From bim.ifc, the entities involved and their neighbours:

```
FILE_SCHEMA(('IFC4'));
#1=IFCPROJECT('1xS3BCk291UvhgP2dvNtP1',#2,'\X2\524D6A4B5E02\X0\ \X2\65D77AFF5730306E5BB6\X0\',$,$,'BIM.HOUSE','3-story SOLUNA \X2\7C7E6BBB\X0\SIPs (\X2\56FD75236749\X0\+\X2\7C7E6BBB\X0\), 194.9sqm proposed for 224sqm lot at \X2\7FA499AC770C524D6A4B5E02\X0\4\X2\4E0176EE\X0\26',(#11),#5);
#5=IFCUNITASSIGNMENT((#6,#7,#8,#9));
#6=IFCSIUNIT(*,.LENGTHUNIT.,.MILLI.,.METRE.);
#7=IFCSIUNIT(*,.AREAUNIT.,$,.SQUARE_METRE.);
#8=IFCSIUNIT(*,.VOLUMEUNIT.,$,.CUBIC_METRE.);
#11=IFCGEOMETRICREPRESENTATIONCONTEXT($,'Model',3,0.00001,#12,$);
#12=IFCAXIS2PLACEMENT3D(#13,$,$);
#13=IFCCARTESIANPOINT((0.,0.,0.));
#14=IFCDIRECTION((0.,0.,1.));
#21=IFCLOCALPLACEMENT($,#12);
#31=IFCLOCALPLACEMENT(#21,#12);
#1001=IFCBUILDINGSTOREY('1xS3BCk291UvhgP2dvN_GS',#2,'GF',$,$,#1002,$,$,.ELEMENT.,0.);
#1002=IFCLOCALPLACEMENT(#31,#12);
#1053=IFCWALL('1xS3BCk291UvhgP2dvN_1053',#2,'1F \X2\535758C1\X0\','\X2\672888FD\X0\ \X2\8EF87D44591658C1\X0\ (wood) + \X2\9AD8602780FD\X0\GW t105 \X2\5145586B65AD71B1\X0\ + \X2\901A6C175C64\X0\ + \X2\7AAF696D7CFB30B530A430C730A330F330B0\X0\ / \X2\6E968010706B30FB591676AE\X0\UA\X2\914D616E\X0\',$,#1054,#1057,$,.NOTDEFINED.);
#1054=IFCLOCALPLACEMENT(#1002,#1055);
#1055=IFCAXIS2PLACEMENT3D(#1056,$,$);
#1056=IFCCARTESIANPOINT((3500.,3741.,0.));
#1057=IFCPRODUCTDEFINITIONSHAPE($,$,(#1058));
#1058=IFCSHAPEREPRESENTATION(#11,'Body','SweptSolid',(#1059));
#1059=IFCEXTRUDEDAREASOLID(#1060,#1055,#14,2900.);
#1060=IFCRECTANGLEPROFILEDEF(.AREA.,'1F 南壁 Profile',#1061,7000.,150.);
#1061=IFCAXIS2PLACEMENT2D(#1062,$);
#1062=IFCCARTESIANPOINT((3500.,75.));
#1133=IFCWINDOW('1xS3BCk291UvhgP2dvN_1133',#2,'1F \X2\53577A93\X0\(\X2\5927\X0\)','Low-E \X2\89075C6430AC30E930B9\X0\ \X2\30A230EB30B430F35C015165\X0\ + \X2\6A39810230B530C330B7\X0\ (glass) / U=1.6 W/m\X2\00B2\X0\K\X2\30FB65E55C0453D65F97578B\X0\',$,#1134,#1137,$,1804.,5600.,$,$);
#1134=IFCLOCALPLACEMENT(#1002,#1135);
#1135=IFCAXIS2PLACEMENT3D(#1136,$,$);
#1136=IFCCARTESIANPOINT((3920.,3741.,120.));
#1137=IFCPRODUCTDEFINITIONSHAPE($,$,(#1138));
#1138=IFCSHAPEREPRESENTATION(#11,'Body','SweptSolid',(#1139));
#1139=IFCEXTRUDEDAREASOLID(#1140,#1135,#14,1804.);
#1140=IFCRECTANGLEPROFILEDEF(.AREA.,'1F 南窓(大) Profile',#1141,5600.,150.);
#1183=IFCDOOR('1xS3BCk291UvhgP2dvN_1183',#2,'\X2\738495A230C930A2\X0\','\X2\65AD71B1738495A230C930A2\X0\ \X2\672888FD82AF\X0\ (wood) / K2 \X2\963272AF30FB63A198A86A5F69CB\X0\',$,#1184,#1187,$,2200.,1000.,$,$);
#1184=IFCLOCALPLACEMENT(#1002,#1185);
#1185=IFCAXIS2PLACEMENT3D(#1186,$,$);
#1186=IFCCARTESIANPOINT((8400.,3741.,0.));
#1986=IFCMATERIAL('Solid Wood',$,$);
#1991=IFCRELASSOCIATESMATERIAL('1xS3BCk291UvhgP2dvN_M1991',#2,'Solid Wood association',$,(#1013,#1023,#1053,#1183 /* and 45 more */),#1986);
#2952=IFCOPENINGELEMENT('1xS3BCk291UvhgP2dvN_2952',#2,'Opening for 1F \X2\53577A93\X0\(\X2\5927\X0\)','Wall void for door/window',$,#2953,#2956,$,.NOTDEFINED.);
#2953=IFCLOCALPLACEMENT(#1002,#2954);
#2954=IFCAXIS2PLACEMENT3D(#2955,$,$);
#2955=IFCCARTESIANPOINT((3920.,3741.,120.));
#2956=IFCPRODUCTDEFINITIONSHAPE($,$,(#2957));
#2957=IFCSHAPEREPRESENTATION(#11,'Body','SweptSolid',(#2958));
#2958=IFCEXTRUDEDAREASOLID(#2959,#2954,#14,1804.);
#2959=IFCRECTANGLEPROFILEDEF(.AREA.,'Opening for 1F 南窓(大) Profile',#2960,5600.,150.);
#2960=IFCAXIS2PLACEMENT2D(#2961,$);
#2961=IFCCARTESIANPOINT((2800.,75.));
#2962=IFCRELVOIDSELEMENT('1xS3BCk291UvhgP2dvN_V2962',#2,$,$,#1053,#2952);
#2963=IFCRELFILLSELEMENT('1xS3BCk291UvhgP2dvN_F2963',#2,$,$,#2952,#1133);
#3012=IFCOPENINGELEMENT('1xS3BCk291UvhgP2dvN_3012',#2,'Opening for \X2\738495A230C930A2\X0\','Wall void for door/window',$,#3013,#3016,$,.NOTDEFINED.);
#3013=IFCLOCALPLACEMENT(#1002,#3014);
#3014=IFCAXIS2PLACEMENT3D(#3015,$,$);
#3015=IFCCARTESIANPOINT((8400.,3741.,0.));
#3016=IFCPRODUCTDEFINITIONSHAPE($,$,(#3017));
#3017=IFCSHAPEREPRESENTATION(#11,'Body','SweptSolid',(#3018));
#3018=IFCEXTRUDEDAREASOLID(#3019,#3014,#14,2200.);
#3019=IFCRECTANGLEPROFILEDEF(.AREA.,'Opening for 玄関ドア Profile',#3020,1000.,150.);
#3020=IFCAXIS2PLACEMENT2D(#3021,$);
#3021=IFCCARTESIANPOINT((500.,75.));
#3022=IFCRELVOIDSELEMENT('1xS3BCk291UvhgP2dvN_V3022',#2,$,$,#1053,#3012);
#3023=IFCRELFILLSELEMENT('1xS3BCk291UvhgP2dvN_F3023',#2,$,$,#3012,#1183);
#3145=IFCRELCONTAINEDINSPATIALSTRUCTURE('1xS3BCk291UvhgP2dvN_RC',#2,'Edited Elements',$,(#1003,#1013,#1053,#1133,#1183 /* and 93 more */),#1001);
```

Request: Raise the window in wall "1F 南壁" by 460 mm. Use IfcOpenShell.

```python
import numpy as np
import ifcopenshell
import ifcopenshell.api.geometry
import ifcopenshell.util.placement
import ifcopenshell.util.unit

model = ifcopenshell.open("bim.ifc")
unit_scale = ifcopenshell.util.unit.calculate_unit_scale(model)

window = model.by_guid("1xS3BCk291UvhgP2dvN_1133")
opening = window.FillsVoids[0].RelatingOpeningElement
dz = 0.46 / unit_scale

shift = np.array([0.0, 0.0, dz])
# The window is not placed relative to its opening, so move both.
for product in (opening, window):
    matrix = ifcopenshell.util.placement.get_local_placement(product.ObjectPlacement)
    matrix[:3, 3] += shift
    ifcopenshell.api.geometry.edit_object_placement(model, product=product, matrix=matrix, is_si=False)

print(f"moved by {dz * unit_scale:+.3f} m")

model.write("bim_updated.ifc")
```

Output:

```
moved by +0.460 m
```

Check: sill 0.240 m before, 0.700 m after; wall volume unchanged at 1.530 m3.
